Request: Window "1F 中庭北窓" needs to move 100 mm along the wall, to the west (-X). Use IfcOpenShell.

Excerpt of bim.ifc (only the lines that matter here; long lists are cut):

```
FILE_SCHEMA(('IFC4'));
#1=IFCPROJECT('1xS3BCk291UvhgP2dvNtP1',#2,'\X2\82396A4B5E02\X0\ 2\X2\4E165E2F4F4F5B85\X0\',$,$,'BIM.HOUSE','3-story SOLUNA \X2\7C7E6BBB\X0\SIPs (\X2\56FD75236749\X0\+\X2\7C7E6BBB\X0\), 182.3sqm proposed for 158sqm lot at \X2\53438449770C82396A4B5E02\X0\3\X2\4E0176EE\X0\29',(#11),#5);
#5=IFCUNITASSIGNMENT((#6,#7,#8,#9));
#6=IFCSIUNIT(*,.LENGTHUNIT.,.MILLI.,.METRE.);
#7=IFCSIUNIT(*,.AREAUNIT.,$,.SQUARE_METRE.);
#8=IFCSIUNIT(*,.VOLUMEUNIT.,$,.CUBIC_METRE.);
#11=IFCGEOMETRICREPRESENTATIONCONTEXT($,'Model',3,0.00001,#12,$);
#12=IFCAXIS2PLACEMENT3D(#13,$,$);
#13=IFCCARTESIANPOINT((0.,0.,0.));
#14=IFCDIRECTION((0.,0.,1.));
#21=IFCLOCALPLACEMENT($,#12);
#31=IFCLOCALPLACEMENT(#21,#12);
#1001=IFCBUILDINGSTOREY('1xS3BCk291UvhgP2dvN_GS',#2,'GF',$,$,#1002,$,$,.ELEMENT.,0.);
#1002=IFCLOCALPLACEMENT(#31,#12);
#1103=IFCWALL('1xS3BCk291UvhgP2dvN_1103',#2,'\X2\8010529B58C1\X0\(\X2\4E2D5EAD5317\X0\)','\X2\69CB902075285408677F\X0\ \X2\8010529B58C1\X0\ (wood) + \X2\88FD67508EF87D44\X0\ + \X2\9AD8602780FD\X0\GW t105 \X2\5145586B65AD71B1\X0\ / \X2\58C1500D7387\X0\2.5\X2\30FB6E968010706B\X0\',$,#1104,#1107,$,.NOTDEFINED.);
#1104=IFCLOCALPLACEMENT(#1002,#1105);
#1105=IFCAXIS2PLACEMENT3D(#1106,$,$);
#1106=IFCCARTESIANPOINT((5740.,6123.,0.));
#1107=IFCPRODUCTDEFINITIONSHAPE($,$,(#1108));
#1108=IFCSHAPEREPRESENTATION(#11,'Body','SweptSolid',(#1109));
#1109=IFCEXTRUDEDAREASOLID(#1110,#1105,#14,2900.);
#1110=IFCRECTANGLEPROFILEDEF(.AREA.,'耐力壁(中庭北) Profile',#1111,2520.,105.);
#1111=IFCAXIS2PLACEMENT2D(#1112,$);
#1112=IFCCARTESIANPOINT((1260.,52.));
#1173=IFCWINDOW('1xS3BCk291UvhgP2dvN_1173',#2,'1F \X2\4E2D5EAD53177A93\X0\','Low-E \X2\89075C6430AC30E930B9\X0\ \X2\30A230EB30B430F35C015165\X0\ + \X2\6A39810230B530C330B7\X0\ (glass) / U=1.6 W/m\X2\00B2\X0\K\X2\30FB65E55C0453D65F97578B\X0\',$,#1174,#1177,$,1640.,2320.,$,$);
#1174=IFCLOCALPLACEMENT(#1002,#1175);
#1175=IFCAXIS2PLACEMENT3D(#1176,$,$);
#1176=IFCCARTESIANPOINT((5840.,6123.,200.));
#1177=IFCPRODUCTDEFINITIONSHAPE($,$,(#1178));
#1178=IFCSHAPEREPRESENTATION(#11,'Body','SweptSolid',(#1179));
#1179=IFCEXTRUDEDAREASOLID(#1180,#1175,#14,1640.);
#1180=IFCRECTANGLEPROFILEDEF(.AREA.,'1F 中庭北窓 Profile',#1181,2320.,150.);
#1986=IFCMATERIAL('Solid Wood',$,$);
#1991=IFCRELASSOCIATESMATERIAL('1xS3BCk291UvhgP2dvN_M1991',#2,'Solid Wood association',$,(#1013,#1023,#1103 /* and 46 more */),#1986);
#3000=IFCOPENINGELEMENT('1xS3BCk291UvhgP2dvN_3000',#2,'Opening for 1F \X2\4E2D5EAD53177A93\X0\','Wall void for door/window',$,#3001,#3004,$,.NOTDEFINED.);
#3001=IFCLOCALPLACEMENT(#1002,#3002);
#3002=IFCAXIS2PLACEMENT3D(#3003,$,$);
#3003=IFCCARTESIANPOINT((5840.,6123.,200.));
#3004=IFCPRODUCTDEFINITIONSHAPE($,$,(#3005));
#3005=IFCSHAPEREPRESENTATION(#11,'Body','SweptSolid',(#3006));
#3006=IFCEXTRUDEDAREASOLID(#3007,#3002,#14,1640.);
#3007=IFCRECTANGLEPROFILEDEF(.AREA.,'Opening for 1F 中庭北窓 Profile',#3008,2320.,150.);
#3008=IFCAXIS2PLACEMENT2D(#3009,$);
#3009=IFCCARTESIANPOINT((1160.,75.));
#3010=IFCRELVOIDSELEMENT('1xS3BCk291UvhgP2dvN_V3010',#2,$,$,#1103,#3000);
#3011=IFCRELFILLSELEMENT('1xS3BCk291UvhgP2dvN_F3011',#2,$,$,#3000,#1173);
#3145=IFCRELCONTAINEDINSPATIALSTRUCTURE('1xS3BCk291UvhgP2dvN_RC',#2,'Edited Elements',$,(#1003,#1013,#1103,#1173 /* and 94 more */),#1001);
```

```python
import ifcopenshell
import ifcopenshell.api.geometry
import ifcopenshell.util.placement

model = ifcopenshell.open("bim.ifc")

window = model.by_guid("1xS3BCk291UvhgP2dvN_1173")
opening = window.FillsVoids[0].RelatingOpeningElement
wall = opening.VoidsElements[0].RelatingBuildingElement

wall_matrix = ifcopenshell.util.placement.get_local_placement(wall.ObjectPlacement)
shift = wall_matrix[:3, 0] * -100.0
before = ifcopenshell.util.placement.get_local_placement(window.ObjectPlacement)[:3, 3].copy()

# The window is not placed relative to its opening, so move both.
for product in (opening, window):
    matrix = ifcopenshell.util.placement.get_local_placement(product.ObjectPlacement)
    matrix[:3, 3] += shift
    ifcopenshell.api.geometry.edit_object_placement(model, product=product, matrix=matrix, is_si=False)

after = ifcopenshell.util.placement.get_local_placement(window.ObjectPlacement)[:3, 3]
print("window moved by", (after - before).round(3) + 0.0)

model.write("bim_v2.ifc")
```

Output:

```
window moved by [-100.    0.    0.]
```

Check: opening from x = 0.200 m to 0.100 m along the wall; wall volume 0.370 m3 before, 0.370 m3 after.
